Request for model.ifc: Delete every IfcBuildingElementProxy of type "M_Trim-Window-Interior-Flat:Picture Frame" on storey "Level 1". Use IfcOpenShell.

First a look at what the model holds.

```python
import ifcopenshell
import ifcopenshell.util.element

model = ifcopenshell.open("model.ifc")
print(model.schema)
storey = next(s for s in model.by_type("IfcBuildingStorey") if s.Name == "Level 1")
proxies = [e for e in ifcopenshell.util.element.get_decomposition(storey) if e.is_a("IfcBuildingElementProxy")]
seen = {}
for e in proxies:
    element_type = ifcopenshell.util.element.get_type(e)
    name = element_type.Name if element_type not in (None, e) else None
    seen[name] = seen.get(name, 0) + 1
for name, count in sorted(seen.items(), key=str):
    print(count, "x", name)
```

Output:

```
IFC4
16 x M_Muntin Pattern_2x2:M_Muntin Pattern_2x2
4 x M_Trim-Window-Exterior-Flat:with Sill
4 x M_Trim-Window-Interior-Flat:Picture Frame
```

```python
import ifcopenshell
import ifcopenshell.api.root
import ifcopenshell.util.element

model = ifcopenshell.open("model.ifc")

storey = next(s for s in model.by_type("IfcBuildingStorey") if s.Name == "Level 1")
proxies = [e for e in ifcopenshell.util.element.get_decomposition(storey) if e.is_a("IfcBuildingElementProxy")]
targets = [e for e in proxies if (t := ifcopenshell.util.element.get_type(e)) not in (None, e) and t.Name == "M_Trim-Window-Interior-Flat:Picture Frame"]

for e in targets:
    ifcopenshell.api.root.remove_product(model, product=e)
print(len(targets), "removed")

model.write("model_v2.ifc")
```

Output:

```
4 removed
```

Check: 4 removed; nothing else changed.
